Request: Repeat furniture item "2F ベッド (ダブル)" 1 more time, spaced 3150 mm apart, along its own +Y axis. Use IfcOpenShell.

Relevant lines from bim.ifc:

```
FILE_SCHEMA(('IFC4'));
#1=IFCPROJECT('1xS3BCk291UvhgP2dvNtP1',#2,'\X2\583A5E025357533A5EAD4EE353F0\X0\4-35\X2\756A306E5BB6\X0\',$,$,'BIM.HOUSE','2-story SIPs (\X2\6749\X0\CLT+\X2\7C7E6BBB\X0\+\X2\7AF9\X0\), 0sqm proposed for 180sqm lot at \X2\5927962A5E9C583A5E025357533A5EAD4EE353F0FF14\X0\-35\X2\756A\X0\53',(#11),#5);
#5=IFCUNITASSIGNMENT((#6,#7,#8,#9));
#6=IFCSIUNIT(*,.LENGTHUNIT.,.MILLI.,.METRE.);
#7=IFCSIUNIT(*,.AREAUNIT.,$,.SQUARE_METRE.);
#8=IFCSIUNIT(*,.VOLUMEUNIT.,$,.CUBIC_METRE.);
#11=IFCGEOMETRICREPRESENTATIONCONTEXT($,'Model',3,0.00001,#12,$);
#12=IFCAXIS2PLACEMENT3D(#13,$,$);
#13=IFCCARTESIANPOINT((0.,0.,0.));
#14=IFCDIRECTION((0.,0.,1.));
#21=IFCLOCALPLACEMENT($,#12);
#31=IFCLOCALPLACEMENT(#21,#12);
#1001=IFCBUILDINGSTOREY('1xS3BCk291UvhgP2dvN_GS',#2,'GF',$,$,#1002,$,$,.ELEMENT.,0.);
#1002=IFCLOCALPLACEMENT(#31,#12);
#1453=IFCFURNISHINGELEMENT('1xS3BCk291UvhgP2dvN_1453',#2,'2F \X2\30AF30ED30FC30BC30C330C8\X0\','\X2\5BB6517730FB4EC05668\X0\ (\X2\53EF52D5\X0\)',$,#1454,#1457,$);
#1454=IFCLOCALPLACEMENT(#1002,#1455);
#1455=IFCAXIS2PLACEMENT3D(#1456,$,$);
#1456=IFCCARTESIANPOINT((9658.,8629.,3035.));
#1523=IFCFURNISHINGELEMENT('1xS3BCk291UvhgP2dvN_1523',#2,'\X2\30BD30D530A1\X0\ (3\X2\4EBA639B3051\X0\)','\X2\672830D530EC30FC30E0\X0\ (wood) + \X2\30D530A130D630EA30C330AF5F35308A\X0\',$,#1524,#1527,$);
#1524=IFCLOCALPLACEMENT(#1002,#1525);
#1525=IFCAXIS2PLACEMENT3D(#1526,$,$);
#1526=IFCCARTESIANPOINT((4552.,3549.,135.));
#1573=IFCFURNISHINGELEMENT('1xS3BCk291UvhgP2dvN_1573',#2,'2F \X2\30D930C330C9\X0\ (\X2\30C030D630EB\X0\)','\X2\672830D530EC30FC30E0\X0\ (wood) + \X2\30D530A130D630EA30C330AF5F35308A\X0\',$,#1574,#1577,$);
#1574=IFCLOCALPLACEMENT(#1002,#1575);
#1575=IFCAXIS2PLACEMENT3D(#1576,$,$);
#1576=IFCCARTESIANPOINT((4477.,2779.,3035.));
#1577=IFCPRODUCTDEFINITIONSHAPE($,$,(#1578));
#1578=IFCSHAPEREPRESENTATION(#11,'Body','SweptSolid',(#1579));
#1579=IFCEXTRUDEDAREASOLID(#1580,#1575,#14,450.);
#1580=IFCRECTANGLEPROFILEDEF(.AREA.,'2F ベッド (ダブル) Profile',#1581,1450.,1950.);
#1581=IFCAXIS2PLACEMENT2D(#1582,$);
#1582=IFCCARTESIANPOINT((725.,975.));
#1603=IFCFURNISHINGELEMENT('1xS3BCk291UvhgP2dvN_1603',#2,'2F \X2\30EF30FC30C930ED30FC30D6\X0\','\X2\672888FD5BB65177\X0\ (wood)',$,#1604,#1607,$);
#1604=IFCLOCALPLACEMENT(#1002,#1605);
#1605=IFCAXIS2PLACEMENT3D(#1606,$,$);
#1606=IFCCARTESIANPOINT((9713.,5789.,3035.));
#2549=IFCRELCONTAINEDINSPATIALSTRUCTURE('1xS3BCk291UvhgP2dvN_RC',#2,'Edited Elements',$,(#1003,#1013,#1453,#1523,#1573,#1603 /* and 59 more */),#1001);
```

```python
import ifcopenshell
import ifcopenshell.api.geometry
import ifcopenshell.api.root
import ifcopenshell.util.element
import ifcopenshell.util.placement
import ifcopenshell.util.unit

model = ifcopenshell.open("bim.ifc")
unit_scale = ifcopenshell.util.unit.calculate_unit_scale(model)


def reuse_history(source, copy):
    """copy_class also copies each property set's owner history, people and application; keep the originals."""
    for rel in copy.IsDefinedBy:
        if rel.is_a("IfcRelDefinesByProperties") and (history := rel.RelatingPropertyDefinition.OwnerHistory):
            rel.RelatingPropertyDefinition.OwnerHistory = source.OwnerHistory
            ifcopenshell.util.element.remove_deep2(model, history)


source = model.by_guid("1xS3BCk291UvhgP2dvN_1573")
base = ifcopenshell.util.placement.get_local_placement(source.ObjectPlacement)
step = base[:3, 1] * 3.15 / unit_scale

for i in range(1, 2):
    copy = ifcopenshell.api.root.copy_class(model, product=source)
    copy.Representation = ifcopenshell.util.element.copy_deep(
        model, source.Representation, exclude=["IfcGeometricRepresentationContext", "IfcRepresentationMap"]
    )
    reuse_history(source, copy)
    matrix = base.copy()
    matrix[:3, 3] += i * step
    print("added at", matrix[:3, 3].round(3) + 0.0)
    ifcopenshell.api.geometry.edit_object_placement(model, product=copy, matrix=matrix, is_si=False)

model.write("bim-out.ifc")
```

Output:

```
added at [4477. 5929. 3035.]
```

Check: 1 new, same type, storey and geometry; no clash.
